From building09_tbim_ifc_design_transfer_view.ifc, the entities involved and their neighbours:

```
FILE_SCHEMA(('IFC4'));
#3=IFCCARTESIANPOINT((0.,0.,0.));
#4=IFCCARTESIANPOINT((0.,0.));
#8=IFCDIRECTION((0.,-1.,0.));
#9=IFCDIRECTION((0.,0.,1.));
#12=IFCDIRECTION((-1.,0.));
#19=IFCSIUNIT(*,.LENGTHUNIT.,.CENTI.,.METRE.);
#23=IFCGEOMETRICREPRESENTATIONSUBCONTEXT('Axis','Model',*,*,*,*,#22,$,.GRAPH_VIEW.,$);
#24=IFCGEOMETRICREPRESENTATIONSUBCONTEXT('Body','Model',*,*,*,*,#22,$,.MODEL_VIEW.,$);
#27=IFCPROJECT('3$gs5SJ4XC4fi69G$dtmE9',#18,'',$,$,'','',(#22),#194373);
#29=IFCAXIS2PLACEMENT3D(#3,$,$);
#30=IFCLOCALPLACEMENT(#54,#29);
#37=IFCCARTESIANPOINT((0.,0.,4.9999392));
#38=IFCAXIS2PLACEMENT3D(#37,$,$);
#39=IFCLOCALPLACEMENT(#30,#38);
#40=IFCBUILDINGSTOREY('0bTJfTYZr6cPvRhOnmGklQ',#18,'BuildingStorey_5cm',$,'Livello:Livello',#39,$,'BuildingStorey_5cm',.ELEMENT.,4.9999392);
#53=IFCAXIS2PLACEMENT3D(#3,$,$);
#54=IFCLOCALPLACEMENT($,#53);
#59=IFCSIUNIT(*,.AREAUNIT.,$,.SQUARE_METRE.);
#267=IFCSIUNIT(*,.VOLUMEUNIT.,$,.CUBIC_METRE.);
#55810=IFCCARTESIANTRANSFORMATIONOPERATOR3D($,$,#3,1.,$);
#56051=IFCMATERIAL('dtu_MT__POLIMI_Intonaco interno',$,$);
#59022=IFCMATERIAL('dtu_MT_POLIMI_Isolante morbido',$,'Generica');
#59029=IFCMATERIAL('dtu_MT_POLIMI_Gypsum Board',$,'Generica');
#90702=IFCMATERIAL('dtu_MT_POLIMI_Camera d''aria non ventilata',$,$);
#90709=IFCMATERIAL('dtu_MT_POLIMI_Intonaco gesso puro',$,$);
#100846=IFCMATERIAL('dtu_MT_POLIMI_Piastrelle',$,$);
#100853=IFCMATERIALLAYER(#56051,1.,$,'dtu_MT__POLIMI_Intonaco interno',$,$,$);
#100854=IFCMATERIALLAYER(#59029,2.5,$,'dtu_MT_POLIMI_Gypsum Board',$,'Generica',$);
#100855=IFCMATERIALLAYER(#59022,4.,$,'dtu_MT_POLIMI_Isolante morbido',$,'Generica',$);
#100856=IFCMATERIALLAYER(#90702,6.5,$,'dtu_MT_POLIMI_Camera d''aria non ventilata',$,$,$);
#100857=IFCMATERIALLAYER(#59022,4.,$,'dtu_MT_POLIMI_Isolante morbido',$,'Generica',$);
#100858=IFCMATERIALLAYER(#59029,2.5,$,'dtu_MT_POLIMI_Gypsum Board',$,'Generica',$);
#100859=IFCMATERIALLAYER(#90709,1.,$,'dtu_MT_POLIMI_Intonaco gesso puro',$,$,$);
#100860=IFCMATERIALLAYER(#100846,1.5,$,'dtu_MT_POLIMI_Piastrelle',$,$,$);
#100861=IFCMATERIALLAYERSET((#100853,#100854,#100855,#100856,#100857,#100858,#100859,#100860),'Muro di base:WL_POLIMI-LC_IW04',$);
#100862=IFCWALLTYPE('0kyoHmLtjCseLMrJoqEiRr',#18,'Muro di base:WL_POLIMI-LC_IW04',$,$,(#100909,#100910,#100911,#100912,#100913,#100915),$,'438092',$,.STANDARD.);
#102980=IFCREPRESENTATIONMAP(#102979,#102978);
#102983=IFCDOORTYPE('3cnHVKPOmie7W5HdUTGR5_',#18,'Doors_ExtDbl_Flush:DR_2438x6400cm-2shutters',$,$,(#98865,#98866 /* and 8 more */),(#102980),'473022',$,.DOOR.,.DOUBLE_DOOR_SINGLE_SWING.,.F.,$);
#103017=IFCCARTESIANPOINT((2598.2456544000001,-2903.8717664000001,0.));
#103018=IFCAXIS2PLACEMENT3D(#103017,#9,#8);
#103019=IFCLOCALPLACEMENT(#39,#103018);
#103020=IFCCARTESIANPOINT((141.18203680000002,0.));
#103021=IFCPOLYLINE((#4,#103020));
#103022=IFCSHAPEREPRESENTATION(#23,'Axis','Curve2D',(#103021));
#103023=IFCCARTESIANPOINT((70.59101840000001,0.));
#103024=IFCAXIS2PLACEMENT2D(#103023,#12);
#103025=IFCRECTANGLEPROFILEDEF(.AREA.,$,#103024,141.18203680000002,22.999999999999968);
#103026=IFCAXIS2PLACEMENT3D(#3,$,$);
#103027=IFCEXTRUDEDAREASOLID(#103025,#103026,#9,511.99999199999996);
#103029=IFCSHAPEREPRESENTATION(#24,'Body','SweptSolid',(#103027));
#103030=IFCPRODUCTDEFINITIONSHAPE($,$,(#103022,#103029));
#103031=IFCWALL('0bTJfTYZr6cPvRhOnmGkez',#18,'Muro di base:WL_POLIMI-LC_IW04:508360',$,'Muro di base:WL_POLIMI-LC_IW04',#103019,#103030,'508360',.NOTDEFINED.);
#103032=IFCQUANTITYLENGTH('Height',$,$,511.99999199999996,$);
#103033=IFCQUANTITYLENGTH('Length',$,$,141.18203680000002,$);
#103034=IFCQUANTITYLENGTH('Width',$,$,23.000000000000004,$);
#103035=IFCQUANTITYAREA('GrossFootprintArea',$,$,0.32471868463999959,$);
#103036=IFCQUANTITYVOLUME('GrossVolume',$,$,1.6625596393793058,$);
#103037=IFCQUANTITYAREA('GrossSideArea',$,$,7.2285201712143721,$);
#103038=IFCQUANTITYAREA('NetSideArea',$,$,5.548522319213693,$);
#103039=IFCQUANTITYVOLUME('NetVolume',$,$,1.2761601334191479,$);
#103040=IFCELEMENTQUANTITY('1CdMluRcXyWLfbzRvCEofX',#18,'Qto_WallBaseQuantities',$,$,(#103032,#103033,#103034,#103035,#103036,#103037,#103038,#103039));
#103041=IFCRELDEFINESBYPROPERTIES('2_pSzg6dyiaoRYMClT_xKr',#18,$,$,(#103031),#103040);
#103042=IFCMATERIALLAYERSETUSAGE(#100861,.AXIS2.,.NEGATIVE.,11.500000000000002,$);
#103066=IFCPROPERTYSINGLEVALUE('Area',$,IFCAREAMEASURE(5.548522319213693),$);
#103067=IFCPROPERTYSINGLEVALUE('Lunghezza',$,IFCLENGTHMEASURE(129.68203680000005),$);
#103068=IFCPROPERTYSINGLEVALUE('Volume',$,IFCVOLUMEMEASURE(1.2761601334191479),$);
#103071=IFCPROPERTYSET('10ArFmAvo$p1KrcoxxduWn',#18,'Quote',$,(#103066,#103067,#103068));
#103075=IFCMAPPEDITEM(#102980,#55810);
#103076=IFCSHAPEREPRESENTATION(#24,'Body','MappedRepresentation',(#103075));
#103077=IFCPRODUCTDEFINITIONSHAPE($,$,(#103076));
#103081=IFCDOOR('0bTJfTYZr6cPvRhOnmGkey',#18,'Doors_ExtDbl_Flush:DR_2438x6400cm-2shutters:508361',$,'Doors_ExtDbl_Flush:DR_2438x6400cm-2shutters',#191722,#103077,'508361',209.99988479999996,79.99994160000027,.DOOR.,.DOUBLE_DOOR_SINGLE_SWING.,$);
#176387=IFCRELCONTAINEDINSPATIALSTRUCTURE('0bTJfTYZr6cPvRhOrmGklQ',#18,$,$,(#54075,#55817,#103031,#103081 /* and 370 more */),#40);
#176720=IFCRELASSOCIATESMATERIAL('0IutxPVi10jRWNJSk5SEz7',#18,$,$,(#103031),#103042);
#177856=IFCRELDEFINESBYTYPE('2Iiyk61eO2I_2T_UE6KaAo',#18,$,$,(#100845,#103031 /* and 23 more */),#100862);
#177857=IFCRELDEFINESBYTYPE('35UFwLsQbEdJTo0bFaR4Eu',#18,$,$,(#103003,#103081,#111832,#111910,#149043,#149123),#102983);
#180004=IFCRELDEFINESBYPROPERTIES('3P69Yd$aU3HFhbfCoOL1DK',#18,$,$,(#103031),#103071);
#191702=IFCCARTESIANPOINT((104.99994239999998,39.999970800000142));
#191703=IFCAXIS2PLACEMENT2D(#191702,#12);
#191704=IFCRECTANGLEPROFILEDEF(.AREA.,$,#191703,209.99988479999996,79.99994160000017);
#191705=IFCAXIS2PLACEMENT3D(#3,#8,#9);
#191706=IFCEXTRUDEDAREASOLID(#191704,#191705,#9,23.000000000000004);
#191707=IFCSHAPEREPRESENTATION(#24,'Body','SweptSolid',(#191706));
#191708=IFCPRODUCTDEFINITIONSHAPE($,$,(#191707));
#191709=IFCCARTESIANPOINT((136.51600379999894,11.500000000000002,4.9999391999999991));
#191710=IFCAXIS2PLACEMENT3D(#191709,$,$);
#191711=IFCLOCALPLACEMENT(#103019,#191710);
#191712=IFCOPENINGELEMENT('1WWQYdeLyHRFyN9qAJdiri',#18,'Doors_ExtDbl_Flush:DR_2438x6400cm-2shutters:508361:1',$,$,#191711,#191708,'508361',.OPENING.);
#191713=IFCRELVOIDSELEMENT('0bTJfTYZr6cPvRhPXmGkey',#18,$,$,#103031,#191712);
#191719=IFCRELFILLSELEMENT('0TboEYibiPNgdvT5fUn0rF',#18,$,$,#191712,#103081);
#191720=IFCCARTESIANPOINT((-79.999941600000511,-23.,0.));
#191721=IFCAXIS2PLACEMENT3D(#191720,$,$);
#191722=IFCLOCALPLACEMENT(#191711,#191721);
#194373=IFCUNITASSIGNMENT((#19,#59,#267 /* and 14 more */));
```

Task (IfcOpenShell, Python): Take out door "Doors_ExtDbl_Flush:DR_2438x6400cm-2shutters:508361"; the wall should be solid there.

```python
import ifcopenshell
import ifcopenshell.api.feature
import ifcopenshell.api.pset
import ifcopenshell.api.root
import ifcopenshell.geom
import ifcopenshell.util.element
import ifcopenshell.util.shape
import ifcopenshell.util.unit

model = ifcopenshell.open("building09_tbim_ifc_design_transfer_view.ifc")
area_scale = ifcopenshell.util.unit.calculate_unit_scale(model, "AREAUNIT")
volume_scale = ifcopenshell.util.unit.calculate_unit_scale(model, "VOLUMEUNIT")
settings = ifcopenshell.geom.settings()


def volume(element):
    """Net volume in cubic metres, openings subtracted."""
    shape = ifcopenshell.geom.create_shape(settings, element)
    return ifcopenshell.util.shape.get_volume(shape.geometry)


door = model.by_guid("0bTJfTYZr6cPvRhOnmGkey")
opening = door.FillsVoids[0].RelatingOpeningElement
wall = opening.VoidsElements[0].RelatingBuildingElement
before = volume(wall)

ifcopenshell.api.root.remove_product(model, product=door)
ifcopenshell.api.feature.remove_feature(model, feature=opening)

after = volume(wall)
thickness = 0.23  # wall thickness in metres

# Update the wall's stored quantities.
qto = model.by_id(ifcopenshell.util.element.get_pset(wall, "Qto_WallBaseQuantities", should_inherit=False)["id"])
ifcopenshell.api.pset.edit_qto(model, qto=qto, properties={
    "NetSideArea": after / thickness / area_scale,
    "NetVolume": after / volume_scale,
})
pset = model.by_id(ifcopenshell.util.element.get_pset(wall, "Quote", should_inherit=False)["id"])
ifcopenshell.api.pset.edit_pset(model, pset=pset, properties={
    "Area": model.create_entity("IfcAreaMeasure", after / thickness / area_scale),
    "Volume": model.create_entity("IfcVolumeMeasure", after / volume_scale),
})

print(f"wall volume {before:.3f} -> {after:.3f} m3")

model.write("building09_tbim_ifc_design_transfer_view_updated.ifc")
```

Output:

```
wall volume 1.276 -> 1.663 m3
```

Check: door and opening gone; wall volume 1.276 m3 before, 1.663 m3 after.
